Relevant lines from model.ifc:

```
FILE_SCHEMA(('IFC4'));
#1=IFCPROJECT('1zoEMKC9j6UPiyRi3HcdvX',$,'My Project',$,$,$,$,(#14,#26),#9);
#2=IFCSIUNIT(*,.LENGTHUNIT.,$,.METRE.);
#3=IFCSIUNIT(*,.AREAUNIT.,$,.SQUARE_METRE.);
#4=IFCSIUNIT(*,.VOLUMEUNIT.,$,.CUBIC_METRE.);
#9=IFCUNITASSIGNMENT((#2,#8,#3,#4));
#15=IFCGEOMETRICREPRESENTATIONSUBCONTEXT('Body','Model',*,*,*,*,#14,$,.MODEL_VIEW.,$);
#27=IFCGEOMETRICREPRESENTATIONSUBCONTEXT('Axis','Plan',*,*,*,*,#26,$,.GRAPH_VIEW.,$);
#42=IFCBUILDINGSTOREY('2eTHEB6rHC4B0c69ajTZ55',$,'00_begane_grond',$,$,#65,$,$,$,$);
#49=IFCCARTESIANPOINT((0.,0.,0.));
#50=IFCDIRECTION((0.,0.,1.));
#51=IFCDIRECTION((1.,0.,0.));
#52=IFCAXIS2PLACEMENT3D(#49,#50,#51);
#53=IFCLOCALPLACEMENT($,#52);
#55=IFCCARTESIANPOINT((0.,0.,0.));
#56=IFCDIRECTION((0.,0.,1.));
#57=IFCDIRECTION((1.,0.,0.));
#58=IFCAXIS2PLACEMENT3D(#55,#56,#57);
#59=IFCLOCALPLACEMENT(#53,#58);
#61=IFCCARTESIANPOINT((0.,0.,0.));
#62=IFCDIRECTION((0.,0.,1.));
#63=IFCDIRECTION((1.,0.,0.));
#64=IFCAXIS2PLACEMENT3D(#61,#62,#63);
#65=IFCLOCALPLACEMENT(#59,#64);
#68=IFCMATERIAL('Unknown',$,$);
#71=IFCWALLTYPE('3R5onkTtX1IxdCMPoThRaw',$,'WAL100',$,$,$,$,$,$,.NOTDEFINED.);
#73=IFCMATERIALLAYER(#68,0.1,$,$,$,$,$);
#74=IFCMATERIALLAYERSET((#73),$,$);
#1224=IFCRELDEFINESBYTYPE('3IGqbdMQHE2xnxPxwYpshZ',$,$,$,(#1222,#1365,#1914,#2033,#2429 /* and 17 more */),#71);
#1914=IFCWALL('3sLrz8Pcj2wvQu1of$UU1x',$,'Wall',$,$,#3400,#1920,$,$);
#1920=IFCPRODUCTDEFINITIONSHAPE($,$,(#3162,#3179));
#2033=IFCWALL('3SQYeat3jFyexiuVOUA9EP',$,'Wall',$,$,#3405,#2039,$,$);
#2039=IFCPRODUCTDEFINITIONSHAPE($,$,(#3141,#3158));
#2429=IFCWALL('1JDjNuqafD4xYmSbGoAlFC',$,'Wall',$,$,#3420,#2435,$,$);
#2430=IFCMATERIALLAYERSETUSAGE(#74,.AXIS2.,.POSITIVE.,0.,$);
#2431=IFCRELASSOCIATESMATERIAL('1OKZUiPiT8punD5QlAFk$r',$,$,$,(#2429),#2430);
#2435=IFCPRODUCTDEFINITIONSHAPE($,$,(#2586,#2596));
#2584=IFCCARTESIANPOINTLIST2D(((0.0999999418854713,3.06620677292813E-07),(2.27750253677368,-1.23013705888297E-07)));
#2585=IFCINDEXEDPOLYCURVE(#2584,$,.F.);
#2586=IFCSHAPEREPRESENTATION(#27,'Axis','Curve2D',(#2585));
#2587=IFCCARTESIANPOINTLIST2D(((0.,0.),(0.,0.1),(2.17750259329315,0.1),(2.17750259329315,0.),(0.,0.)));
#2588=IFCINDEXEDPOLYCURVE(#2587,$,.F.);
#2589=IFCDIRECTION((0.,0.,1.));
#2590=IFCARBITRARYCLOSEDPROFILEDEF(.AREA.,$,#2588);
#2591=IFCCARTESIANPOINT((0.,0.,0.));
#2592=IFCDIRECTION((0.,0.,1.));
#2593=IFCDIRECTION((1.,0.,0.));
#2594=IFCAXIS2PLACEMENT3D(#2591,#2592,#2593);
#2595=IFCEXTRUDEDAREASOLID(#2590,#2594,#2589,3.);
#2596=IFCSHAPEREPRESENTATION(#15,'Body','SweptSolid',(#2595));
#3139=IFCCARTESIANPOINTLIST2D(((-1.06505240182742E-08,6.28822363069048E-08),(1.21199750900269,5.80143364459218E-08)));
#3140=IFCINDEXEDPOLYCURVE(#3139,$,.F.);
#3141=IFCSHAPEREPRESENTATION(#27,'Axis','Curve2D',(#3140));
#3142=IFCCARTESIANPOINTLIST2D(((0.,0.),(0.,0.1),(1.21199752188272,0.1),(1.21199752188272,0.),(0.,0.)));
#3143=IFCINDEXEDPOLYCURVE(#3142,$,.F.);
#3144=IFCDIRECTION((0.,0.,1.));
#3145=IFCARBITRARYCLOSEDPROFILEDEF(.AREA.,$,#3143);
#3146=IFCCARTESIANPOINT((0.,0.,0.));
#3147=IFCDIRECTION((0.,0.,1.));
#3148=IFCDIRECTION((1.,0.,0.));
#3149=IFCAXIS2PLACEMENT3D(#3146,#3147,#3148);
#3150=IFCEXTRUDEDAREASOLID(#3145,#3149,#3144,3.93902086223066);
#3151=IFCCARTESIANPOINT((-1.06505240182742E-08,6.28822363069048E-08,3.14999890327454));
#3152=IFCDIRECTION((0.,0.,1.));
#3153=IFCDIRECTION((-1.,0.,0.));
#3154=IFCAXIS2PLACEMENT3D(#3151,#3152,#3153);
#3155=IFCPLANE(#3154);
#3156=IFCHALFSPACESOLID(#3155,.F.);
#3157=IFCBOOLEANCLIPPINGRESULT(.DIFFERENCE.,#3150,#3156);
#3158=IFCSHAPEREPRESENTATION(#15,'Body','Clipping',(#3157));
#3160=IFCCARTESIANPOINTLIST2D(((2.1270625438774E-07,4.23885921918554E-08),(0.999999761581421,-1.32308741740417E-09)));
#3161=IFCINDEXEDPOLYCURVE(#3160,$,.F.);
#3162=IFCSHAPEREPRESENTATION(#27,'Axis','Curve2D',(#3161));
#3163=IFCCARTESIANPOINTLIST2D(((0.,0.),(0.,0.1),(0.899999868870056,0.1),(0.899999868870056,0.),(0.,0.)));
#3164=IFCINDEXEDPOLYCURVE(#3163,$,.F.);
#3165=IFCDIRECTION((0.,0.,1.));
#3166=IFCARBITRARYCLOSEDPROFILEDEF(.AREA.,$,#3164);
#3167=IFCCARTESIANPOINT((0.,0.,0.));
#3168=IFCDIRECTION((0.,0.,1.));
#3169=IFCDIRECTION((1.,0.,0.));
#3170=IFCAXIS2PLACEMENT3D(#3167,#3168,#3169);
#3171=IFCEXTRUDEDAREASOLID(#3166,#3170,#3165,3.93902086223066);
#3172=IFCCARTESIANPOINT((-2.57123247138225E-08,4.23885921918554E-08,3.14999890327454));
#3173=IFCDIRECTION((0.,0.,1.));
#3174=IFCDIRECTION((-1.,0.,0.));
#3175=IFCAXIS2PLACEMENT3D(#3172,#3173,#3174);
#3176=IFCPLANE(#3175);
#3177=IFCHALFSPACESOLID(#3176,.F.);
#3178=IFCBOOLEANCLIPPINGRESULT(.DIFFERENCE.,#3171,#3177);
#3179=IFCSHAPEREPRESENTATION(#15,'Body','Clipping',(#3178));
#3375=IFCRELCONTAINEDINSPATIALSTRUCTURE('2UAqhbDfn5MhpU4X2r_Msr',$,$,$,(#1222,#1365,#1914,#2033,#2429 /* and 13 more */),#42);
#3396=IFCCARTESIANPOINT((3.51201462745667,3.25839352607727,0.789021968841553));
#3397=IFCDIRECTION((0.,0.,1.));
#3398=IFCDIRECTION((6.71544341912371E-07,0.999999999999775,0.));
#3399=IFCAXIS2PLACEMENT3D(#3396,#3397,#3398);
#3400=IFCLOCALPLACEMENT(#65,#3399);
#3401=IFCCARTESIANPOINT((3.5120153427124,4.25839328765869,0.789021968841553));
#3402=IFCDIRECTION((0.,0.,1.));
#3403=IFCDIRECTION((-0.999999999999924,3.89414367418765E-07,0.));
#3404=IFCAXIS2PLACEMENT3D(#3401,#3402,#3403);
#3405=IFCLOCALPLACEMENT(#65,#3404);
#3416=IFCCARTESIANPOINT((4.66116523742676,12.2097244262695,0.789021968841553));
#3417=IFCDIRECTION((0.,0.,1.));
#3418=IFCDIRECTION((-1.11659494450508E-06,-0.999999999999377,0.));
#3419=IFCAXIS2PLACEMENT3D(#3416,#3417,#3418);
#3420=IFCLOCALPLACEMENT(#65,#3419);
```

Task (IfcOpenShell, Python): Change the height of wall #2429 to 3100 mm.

```python
import ifcopenshell
import ifcopenshell.geom
import ifcopenshell.util.representation
import ifcopenshell.util.shape

model = ifcopenshell.open("model.ifc")
settings = ifcopenshell.geom.settings()


def volume(element):
    """Net volume in cubic metres, openings subtracted."""
    shape = ifcopenshell.geom.create_shape(settings, element)
    return ifcopenshell.util.shape.get_volume(shape.geometry)


wall = model.by_guid("1JDjNuqafD4xYmSbGoAlFC")
before = volume(wall)

body = ifcopenshell.util.representation.get_representation(wall, "Model", "Body")
solid = body.Items[0]
old_height = solid.Depth
solid.Depth = 3.1
after = volume(wall)

print(f"height {old_height:g} -> {solid.Depth:g}, volume {before:.3f} -> {after:.3f} m3")

model.write("model_rev.ifc")
```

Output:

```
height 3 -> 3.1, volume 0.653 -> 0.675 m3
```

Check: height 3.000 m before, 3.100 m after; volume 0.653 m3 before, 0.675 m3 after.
